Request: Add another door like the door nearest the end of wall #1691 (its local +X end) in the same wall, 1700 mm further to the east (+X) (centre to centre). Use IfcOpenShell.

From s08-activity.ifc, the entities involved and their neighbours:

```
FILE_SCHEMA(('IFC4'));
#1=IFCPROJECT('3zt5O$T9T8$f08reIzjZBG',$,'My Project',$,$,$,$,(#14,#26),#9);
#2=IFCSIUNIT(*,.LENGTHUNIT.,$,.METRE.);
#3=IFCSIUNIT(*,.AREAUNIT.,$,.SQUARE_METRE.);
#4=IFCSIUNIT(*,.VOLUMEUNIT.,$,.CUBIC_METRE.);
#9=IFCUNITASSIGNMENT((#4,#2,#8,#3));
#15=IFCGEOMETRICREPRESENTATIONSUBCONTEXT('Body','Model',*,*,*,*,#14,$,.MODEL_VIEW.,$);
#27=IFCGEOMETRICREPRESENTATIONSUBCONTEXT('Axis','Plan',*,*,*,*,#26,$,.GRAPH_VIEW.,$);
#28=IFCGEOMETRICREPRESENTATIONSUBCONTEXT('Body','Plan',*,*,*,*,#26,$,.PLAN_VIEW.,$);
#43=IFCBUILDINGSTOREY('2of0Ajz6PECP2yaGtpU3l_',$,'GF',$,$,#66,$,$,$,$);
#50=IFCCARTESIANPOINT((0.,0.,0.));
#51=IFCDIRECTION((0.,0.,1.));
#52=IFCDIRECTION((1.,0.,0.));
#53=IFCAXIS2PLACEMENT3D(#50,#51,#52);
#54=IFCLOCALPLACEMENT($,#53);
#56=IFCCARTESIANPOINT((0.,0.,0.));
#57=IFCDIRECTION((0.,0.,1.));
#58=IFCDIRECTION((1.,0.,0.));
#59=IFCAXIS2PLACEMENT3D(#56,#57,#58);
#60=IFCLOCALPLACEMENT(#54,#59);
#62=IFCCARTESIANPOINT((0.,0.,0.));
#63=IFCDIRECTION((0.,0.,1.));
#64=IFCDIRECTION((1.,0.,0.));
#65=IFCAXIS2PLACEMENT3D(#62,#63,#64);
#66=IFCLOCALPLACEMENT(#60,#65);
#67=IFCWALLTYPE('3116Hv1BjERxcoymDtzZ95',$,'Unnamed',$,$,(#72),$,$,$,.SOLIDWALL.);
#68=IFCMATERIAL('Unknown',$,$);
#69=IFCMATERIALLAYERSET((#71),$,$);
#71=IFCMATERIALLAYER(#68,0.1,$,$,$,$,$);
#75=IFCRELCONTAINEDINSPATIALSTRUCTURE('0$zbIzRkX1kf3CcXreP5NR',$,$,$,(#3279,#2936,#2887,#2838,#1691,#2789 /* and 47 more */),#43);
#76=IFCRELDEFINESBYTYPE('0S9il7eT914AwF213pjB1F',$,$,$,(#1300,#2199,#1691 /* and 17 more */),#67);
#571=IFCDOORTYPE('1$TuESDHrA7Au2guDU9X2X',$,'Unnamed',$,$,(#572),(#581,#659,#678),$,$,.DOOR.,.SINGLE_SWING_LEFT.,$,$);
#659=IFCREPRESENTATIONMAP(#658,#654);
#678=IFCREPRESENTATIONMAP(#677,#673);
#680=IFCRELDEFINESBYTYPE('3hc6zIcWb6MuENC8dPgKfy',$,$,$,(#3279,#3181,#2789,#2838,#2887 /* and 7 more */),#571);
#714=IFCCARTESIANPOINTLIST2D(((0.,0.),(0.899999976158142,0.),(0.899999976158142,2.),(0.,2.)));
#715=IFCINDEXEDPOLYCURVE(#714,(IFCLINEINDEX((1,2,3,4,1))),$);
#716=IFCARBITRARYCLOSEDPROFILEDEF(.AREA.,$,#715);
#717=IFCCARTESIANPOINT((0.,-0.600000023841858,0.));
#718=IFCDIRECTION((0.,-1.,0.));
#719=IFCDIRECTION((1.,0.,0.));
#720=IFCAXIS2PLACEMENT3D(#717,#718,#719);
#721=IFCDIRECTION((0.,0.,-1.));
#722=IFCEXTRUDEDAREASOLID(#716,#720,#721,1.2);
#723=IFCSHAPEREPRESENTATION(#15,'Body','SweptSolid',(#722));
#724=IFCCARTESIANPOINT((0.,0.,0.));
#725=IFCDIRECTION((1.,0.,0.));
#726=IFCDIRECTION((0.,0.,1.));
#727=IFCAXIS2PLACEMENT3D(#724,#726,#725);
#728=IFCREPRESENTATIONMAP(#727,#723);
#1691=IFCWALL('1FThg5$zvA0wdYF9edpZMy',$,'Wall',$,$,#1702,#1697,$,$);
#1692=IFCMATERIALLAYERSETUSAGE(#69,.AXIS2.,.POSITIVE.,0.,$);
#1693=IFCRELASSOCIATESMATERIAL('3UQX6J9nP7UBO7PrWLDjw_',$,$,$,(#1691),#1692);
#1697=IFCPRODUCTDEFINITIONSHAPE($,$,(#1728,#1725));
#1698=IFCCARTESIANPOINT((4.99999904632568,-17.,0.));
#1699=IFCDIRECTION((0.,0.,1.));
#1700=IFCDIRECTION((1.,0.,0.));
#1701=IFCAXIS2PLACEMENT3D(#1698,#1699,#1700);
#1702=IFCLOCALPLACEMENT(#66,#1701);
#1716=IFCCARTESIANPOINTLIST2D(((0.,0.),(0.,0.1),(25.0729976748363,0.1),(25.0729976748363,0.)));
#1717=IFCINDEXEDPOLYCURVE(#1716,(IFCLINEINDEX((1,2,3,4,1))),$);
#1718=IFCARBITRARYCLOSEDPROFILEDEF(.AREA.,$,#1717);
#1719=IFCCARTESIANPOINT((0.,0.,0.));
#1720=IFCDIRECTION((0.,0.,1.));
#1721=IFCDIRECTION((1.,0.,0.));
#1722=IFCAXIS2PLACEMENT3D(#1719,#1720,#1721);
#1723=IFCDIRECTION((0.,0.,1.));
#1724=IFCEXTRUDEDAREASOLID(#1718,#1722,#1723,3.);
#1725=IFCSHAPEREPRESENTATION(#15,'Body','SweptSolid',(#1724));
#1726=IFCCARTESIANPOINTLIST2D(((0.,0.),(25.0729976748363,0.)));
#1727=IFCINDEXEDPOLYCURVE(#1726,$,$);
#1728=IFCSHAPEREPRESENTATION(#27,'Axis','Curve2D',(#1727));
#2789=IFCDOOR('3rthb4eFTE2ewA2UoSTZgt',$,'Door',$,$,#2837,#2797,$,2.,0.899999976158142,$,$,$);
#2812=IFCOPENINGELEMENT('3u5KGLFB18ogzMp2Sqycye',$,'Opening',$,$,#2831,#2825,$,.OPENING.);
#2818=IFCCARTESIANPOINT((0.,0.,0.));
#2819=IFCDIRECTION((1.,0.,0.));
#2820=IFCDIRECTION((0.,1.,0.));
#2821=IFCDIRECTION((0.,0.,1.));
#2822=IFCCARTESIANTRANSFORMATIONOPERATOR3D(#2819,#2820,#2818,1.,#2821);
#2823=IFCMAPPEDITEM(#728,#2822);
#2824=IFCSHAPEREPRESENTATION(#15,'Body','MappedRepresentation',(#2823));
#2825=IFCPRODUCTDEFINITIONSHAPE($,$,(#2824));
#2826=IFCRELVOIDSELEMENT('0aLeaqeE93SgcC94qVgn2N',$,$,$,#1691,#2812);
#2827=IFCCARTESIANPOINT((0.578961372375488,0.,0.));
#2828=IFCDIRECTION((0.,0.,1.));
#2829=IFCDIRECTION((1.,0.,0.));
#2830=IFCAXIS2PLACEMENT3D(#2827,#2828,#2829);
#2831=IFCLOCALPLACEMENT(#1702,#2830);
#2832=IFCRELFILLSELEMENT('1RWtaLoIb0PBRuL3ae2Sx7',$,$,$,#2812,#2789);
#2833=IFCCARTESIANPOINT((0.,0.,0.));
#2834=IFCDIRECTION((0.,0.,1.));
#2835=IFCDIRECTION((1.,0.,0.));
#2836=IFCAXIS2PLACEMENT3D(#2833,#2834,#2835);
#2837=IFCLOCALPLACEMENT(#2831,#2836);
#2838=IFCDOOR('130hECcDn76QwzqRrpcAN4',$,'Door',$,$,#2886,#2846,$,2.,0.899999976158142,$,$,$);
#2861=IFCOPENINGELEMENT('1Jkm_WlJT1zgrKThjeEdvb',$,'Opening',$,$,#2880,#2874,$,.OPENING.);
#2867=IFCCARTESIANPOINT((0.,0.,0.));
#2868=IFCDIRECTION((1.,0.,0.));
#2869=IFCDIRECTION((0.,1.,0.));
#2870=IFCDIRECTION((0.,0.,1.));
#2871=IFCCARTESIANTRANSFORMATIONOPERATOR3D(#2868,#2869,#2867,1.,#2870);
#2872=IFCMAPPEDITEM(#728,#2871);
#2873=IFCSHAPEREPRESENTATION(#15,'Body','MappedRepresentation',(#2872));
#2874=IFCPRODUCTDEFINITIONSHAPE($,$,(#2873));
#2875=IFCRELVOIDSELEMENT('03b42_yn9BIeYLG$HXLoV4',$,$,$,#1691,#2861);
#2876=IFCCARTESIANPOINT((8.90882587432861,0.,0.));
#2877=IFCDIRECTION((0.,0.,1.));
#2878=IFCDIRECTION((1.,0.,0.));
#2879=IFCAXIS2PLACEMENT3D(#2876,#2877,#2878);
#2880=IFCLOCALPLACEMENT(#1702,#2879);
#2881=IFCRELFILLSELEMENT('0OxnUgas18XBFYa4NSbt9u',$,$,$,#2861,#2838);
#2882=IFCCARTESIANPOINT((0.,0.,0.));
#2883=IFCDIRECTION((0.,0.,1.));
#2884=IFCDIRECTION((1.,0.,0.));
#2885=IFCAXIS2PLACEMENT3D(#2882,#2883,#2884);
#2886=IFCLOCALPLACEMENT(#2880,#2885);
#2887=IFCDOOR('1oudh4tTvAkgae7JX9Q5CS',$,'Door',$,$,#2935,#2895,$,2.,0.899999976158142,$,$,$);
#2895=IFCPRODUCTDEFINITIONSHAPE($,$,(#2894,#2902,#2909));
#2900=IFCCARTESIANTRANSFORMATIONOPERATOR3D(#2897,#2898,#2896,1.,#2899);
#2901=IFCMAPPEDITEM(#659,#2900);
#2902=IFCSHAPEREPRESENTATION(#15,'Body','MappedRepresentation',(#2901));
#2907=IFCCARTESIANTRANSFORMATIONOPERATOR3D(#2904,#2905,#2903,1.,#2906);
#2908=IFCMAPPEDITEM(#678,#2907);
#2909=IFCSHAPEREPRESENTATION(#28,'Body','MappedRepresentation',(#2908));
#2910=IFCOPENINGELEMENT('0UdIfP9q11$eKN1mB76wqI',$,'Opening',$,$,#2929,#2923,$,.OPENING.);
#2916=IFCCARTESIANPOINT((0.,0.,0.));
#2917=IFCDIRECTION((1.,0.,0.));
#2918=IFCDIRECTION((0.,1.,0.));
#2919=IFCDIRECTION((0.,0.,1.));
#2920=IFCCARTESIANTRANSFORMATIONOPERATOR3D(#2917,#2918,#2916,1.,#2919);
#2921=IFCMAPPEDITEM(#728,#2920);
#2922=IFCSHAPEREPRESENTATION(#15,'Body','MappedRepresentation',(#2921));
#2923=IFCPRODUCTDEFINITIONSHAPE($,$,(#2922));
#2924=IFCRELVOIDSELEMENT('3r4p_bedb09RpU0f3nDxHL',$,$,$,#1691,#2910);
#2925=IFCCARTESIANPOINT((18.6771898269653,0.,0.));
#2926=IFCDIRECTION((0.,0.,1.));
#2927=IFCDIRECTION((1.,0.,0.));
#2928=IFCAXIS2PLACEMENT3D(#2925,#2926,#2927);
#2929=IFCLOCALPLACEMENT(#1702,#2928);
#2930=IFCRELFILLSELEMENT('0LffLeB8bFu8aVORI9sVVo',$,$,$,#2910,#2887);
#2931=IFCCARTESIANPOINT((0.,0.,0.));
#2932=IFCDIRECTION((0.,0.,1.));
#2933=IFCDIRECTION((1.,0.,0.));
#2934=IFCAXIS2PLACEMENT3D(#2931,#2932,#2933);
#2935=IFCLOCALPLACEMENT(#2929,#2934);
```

```python
import ifcopenshell
import ifcopenshell.api.feature
import ifcopenshell.api.geometry
import ifcopenshell.api.root
import ifcopenshell.geom
import ifcopenshell.util.element
import ifcopenshell.util.placement
import ifcopenshell.util.shape

model = ifcopenshell.open("s08-activity.ifc")
settings = ifcopenshell.geom.settings()


def volume(element):
    """Net volume in cubic metres, openings subtracted."""
    shape = ifcopenshell.geom.create_shape(settings, element)
    return ifcopenshell.util.shape.get_volume(shape.geometry)


door = model.by_guid("1oudh4tTvAkgae7JX9Q5CS")
opening = door.FillsVoids[0].RelatingOpeningElement
wall = opening.VoidsElements[0].RelatingBuildingElement
before = volume(wall)
shift = ifcopenshell.util.placement.get_local_placement(wall.ObjectPlacement)[:3, 0] * 1.7

# copy_class copies the void relationship, type, container and properties, but no geometry.
new_opening = ifcopenshell.api.root.copy_class(model, product=opening)
new_opening.Representation = ifcopenshell.util.element.copy_deep(
    model, opening.Representation, exclude=["IfcGeometricRepresentationContext", "IfcRepresentationMap"]
)
new_door = ifcopenshell.api.root.copy_class(model, product=door)
new_door.Representation = ifcopenshell.util.element.copy_deep(
    model, door.Representation, exclude=["IfcGeometricRepresentationContext", "IfcRepresentationMap"]
)
ifcopenshell.api.feature.add_filling(model, opening=new_opening, element=new_door)

for old, new in ((opening, new_opening), (door, new_door)):
    matrix = ifcopenshell.util.placement.get_local_placement(old.ObjectPlacement)
    matrix[:3, 3] += shift
    ifcopenshell.api.geometry.edit_object_placement(model, product=new, matrix=matrix, is_si=False)

after = volume(wall)

print(f"wall volume {before:.3f} -> {after:.3f} m3")

model.write("s08-activity_rev.ifc")
```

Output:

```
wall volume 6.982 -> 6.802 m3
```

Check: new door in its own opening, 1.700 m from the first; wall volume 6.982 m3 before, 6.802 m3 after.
